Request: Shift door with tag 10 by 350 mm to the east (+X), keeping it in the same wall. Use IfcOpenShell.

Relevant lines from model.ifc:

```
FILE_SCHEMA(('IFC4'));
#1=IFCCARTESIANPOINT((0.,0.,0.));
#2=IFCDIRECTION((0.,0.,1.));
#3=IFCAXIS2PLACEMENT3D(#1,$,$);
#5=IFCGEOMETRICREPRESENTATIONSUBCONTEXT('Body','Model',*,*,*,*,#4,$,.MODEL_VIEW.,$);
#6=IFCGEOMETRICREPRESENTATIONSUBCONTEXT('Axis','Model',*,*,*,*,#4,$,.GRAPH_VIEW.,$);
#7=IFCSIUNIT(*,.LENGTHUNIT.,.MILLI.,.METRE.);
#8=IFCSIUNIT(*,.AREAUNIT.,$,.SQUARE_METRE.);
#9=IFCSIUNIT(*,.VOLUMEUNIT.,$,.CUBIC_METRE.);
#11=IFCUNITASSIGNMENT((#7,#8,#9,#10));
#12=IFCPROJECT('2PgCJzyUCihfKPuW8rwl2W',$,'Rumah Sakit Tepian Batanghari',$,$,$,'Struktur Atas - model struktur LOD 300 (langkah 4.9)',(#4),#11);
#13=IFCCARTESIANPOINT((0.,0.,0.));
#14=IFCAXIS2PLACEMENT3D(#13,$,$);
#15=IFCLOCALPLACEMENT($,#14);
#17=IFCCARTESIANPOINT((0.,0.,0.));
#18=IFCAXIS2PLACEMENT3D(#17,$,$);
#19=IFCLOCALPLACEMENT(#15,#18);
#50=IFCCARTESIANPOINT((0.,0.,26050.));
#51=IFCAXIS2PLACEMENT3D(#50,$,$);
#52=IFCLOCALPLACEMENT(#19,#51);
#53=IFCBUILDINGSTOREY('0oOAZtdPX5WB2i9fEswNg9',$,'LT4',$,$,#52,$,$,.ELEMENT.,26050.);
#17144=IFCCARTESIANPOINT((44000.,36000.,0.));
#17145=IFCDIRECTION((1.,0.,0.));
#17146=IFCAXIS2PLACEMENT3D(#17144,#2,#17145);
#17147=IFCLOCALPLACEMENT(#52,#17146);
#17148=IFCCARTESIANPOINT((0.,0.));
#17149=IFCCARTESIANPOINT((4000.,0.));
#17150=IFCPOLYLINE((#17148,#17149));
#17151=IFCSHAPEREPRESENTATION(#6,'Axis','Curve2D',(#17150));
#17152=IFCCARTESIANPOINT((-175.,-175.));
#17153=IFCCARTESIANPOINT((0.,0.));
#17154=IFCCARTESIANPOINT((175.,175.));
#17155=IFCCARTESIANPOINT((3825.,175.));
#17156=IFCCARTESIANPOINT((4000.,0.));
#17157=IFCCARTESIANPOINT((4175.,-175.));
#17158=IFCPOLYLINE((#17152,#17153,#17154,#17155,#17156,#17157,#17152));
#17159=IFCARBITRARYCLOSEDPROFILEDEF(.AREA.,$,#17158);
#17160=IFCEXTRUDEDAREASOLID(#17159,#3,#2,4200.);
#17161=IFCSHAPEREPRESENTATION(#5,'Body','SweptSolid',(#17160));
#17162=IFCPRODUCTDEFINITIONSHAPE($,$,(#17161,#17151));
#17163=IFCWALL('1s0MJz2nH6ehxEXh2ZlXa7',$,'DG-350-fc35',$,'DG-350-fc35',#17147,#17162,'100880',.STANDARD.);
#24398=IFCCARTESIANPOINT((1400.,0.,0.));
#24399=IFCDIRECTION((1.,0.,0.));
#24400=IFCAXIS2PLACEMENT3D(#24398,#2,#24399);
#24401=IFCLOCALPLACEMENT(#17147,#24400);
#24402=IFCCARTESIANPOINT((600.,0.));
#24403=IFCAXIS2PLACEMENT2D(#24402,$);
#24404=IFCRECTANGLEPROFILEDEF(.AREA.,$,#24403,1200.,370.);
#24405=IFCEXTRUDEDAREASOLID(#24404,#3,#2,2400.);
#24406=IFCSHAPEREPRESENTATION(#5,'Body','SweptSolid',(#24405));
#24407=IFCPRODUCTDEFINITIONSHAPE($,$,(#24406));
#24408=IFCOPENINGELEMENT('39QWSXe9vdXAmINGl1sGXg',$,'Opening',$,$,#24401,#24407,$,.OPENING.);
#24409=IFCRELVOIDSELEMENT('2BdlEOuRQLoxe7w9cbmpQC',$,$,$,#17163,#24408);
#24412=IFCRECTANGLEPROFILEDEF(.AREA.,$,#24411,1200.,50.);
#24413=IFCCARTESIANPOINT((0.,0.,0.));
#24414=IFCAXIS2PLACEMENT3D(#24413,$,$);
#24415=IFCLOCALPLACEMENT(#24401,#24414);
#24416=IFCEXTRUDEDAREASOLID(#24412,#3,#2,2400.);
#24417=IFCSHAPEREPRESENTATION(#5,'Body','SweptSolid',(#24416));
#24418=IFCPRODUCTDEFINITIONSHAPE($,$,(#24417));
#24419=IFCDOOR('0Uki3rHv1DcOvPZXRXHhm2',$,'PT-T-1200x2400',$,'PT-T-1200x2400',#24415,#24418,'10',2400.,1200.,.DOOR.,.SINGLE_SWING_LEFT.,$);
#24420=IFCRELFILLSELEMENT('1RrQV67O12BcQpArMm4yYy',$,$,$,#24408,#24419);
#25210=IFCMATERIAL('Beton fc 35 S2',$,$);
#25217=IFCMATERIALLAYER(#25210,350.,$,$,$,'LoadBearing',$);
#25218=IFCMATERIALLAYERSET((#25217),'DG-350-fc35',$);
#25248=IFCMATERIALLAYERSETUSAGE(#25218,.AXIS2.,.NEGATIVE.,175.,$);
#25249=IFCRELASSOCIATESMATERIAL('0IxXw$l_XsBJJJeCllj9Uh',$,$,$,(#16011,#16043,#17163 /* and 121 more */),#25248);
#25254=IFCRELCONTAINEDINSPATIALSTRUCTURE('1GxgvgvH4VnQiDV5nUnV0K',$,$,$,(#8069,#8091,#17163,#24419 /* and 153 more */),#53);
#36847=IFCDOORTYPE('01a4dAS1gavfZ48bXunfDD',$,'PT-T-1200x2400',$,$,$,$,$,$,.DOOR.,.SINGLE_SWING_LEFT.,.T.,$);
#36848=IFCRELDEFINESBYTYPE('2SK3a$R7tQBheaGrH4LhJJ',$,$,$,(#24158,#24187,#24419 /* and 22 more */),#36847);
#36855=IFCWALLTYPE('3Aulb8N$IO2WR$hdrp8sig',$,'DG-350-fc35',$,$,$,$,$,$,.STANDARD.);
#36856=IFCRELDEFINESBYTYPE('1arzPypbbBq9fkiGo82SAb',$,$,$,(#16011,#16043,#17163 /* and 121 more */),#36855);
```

```python
import ifcopenshell
import ifcopenshell.api.geometry
import ifcopenshell.util.placement
import ifcopenshell.util.unit

model = ifcopenshell.open("model.ifc")
unit_scale = ifcopenshell.util.unit.calculate_unit_scale(model)

door = model.by_guid("0Uki3rHv1DcOvPZXRXHhm2")
opening = door.FillsVoids[0].RelatingOpeningElement
wall = opening.VoidsElements[0].RelatingBuildingElement

wall_matrix = ifcopenshell.util.placement.get_local_placement(wall.ObjectPlacement)
shift = wall_matrix[:3, 0] * 0.35 / unit_scale
before = ifcopenshell.util.placement.get_local_placement(door.ObjectPlacement)[:3, 3].copy()

# The door is placed relative to its opening, so it follows when the opening moves.
matrix = ifcopenshell.util.placement.get_local_placement(opening.ObjectPlacement)
matrix[:3, 3] += shift
ifcopenshell.api.geometry.edit_object_placement(
    model, product=opening, matrix=matrix, is_si=False, should_transform_children=True
)

after = ifcopenshell.util.placement.get_local_placement(door.ObjectPlacement)[:3, 3]
print("door moved by", (after - before).round(3) + 0.0)

model.write("model_edited.ifc")
```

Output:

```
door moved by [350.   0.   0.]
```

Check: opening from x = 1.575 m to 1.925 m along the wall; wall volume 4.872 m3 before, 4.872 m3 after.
